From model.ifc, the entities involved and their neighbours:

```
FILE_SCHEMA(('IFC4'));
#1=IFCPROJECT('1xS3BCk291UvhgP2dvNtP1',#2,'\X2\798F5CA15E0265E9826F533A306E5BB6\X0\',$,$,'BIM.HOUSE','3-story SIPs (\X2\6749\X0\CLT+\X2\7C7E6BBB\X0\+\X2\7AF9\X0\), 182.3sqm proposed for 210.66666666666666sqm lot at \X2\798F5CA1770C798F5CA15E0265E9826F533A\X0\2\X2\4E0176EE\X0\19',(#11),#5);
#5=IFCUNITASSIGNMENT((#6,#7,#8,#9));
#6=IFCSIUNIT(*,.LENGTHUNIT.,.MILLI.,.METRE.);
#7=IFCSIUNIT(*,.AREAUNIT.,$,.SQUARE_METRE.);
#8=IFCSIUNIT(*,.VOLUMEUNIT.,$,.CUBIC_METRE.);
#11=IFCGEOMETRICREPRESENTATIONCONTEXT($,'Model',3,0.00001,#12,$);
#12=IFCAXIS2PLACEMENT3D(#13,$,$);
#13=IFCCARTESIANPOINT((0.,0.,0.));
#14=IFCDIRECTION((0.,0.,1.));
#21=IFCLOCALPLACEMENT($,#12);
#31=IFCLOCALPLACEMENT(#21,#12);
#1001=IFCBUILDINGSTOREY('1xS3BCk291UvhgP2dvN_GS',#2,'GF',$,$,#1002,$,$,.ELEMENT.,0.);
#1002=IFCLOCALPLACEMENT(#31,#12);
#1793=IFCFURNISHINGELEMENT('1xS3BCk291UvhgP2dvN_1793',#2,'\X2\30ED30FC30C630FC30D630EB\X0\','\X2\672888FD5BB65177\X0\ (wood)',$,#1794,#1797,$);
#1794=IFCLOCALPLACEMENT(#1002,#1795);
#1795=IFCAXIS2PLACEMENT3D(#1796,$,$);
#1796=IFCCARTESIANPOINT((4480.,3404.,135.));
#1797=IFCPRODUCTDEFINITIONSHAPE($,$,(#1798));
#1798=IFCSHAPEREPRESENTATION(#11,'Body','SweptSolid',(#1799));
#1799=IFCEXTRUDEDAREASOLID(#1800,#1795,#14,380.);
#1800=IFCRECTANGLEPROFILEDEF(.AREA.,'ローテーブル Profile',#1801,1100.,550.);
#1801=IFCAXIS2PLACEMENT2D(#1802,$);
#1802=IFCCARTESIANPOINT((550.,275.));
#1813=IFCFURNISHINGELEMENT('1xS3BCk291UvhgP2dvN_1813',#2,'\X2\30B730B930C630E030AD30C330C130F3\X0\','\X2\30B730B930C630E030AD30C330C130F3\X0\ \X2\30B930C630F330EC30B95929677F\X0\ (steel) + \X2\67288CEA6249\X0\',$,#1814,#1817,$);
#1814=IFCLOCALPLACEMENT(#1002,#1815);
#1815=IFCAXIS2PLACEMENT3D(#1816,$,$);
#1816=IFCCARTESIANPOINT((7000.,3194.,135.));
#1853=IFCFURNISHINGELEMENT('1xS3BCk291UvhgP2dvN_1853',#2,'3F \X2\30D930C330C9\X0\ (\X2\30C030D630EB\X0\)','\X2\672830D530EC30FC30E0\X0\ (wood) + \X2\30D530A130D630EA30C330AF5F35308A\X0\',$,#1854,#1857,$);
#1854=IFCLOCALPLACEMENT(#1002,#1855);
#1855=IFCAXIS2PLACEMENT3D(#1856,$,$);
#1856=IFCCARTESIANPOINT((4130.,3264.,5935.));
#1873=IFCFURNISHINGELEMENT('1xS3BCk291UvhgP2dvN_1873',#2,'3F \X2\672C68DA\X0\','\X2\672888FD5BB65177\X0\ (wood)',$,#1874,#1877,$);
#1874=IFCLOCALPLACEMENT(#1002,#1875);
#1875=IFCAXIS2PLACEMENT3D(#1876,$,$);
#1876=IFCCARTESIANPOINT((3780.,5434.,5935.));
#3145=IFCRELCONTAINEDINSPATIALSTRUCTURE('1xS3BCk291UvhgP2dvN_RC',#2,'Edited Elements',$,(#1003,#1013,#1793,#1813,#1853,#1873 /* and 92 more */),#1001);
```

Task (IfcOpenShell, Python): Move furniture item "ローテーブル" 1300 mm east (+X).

```python
import ifcopenshell
import ifcopenshell.api.geometry
import ifcopenshell.util.placement
import ifcopenshell.util.unit

model = ifcopenshell.open("model.ifc")
unit_scale = ifcopenshell.util.unit.calculate_unit_scale(model)

item = model.by_id(1793)
matrix = ifcopenshell.util.placement.get_local_placement(item.ObjectPlacement)
matrix[0, 3] += 1.3 / unit_scale
ifcopenshell.api.geometry.edit_object_placement(model, product=item, matrix=matrix, is_si=False)

print(ifcopenshell.util.placement.get_local_placement(item.ObjectPlacement).round(3) + 0.0)

model.write("model_updated.ifc")
```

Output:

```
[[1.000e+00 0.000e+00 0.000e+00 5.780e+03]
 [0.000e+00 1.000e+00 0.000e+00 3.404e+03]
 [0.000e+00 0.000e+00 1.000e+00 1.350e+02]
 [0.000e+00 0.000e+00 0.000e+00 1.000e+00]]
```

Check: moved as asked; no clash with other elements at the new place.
